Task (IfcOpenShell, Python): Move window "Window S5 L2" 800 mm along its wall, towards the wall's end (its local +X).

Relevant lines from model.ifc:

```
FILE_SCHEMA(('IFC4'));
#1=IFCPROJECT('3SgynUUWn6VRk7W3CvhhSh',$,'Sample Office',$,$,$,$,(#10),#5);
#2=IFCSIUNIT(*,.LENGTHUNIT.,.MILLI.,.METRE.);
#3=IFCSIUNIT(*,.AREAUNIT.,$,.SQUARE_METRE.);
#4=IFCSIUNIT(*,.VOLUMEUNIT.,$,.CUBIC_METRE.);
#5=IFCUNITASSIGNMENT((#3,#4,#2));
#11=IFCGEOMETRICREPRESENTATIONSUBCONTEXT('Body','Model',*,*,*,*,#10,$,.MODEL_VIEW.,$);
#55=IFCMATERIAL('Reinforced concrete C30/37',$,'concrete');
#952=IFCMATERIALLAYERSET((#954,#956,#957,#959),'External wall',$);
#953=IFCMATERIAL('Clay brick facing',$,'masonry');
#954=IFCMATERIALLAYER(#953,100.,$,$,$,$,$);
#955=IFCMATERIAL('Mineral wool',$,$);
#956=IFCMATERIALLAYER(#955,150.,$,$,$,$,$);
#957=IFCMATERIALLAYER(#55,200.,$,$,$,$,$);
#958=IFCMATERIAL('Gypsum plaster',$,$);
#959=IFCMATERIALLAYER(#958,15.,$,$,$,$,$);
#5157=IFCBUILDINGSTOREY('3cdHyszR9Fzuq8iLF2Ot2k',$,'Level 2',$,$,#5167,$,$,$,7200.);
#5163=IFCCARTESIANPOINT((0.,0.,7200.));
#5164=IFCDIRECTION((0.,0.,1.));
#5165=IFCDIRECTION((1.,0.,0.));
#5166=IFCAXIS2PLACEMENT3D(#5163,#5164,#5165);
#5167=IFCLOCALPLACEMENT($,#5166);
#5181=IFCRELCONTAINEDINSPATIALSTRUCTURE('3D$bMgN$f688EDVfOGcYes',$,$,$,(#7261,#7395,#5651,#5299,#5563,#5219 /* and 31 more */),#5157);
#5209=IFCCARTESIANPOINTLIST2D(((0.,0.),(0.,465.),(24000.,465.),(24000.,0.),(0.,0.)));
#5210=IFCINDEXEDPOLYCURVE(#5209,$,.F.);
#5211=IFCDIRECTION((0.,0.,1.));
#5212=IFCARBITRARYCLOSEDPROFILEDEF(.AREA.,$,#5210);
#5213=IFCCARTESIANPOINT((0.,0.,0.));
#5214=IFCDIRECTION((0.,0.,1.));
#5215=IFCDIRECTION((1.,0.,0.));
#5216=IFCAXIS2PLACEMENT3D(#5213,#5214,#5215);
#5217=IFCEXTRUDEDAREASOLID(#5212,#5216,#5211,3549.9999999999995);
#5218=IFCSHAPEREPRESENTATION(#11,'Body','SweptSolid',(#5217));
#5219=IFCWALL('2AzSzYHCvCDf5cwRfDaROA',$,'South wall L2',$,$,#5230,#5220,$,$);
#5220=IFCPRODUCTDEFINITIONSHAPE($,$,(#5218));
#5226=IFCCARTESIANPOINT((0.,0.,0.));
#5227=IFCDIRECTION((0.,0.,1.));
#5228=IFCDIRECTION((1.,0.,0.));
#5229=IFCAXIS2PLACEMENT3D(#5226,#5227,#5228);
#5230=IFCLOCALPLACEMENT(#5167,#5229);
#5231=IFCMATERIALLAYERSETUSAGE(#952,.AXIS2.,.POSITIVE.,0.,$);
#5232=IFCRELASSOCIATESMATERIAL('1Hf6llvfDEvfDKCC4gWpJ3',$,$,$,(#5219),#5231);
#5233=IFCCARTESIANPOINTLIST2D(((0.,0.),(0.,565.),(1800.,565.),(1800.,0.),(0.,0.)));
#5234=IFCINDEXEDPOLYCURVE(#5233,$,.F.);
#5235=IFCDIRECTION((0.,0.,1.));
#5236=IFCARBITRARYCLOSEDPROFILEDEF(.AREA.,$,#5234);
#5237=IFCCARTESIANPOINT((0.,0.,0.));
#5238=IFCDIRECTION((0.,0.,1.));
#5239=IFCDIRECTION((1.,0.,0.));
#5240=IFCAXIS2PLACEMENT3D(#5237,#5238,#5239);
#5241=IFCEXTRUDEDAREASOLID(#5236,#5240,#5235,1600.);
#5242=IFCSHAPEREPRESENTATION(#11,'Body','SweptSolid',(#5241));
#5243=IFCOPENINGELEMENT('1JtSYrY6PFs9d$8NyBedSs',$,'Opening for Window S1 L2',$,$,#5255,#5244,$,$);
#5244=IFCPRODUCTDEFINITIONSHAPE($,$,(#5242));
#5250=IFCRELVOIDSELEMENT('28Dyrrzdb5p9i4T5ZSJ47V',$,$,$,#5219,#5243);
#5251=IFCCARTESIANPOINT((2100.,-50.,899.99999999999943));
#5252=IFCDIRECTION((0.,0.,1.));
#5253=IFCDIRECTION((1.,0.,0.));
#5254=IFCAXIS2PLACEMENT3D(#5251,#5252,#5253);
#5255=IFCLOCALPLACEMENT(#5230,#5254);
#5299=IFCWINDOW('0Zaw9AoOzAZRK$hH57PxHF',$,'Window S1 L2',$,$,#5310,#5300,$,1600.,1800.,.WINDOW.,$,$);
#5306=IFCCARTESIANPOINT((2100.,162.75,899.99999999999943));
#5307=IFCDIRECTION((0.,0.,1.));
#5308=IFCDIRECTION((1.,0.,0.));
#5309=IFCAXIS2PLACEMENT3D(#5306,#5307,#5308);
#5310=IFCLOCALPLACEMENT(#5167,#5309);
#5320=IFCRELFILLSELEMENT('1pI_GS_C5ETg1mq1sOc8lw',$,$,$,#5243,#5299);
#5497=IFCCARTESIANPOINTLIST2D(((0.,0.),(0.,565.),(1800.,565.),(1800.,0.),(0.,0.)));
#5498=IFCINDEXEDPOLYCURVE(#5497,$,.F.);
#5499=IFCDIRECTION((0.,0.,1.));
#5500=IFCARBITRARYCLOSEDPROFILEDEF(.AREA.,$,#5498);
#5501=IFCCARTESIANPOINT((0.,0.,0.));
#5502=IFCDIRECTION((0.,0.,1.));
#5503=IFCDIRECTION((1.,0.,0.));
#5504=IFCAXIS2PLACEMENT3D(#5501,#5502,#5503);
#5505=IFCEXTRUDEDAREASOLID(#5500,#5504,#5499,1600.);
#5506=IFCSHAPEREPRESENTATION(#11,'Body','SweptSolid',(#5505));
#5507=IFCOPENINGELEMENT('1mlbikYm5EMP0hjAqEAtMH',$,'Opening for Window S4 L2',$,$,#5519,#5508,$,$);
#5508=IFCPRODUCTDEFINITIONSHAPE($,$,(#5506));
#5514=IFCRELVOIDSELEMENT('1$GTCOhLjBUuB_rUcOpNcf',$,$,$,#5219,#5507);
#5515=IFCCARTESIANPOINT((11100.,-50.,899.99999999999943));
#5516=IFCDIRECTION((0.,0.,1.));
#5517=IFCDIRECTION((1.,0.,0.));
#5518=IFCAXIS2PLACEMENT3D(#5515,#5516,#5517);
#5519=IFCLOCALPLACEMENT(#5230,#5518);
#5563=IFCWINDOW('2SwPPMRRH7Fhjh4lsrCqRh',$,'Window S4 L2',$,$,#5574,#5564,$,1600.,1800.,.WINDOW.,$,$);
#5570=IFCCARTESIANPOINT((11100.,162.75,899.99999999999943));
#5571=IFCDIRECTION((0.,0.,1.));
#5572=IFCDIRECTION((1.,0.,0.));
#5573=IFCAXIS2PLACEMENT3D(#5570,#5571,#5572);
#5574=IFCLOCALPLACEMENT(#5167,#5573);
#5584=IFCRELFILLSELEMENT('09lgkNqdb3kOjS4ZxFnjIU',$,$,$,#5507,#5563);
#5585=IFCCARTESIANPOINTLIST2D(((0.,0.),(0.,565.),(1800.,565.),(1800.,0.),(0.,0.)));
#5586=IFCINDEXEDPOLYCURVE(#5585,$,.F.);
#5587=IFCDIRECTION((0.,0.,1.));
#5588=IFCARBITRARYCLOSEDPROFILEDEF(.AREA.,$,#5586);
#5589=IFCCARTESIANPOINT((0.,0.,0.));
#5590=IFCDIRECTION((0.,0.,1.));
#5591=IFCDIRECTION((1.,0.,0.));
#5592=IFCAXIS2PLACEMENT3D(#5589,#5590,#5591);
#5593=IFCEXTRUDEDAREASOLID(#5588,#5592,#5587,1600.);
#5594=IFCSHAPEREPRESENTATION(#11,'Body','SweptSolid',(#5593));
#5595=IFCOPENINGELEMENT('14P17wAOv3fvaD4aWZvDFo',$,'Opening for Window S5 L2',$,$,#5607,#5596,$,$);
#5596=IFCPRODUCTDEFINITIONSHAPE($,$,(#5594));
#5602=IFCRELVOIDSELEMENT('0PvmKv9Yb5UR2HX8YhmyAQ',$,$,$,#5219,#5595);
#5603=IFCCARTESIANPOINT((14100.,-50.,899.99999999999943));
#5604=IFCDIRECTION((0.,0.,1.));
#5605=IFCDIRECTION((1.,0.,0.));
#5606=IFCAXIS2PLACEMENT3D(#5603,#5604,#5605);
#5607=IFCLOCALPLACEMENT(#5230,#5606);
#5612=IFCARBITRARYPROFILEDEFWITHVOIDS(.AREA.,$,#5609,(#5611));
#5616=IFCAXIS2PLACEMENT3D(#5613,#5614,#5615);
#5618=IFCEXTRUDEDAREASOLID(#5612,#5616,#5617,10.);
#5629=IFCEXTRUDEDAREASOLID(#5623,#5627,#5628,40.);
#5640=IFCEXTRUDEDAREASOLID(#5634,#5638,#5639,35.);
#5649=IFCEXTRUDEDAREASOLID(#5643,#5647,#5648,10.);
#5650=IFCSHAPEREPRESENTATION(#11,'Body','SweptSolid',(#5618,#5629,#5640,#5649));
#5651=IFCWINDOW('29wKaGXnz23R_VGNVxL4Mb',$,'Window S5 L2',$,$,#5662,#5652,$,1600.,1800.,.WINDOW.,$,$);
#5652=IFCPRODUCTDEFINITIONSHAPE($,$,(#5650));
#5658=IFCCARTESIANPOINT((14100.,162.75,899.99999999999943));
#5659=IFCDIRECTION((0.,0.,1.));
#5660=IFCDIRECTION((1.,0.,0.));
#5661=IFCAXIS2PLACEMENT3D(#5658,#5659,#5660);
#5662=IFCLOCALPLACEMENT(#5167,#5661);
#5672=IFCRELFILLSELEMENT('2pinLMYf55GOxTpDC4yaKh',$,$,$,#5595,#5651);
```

```python
import ifcopenshell
import ifcopenshell.api.geometry
import ifcopenshell.util.placement

model = ifcopenshell.open("model.ifc")

window = model.by_id(5651)
opening = window.FillsVoids[0].RelatingOpeningElement
wall = opening.VoidsElements[0].RelatingBuildingElement

wall_matrix = ifcopenshell.util.placement.get_local_placement(wall.ObjectPlacement)
shift = wall_matrix[:3, 0] * 800.0
before = ifcopenshell.util.placement.get_local_placement(window.ObjectPlacement)[:3, 3].copy()

# The window is not placed relative to its opening, so move both.
for product in (opening, window):
    matrix = ifcopenshell.util.placement.get_local_placement(product.ObjectPlacement)
    matrix[:3, 3] += shift
    ifcopenshell.api.geometry.edit_object_placement(model, product=product, matrix=matrix, is_si=False)

after = ifcopenshell.util.placement.get_local_placement(window.ObjectPlacement)[:3, 3]
print("window moved by", (after - before).round(3) + 0.0)

model.write("model_rev.ifc")
```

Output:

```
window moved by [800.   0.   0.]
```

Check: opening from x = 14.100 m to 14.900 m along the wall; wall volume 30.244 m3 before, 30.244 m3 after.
